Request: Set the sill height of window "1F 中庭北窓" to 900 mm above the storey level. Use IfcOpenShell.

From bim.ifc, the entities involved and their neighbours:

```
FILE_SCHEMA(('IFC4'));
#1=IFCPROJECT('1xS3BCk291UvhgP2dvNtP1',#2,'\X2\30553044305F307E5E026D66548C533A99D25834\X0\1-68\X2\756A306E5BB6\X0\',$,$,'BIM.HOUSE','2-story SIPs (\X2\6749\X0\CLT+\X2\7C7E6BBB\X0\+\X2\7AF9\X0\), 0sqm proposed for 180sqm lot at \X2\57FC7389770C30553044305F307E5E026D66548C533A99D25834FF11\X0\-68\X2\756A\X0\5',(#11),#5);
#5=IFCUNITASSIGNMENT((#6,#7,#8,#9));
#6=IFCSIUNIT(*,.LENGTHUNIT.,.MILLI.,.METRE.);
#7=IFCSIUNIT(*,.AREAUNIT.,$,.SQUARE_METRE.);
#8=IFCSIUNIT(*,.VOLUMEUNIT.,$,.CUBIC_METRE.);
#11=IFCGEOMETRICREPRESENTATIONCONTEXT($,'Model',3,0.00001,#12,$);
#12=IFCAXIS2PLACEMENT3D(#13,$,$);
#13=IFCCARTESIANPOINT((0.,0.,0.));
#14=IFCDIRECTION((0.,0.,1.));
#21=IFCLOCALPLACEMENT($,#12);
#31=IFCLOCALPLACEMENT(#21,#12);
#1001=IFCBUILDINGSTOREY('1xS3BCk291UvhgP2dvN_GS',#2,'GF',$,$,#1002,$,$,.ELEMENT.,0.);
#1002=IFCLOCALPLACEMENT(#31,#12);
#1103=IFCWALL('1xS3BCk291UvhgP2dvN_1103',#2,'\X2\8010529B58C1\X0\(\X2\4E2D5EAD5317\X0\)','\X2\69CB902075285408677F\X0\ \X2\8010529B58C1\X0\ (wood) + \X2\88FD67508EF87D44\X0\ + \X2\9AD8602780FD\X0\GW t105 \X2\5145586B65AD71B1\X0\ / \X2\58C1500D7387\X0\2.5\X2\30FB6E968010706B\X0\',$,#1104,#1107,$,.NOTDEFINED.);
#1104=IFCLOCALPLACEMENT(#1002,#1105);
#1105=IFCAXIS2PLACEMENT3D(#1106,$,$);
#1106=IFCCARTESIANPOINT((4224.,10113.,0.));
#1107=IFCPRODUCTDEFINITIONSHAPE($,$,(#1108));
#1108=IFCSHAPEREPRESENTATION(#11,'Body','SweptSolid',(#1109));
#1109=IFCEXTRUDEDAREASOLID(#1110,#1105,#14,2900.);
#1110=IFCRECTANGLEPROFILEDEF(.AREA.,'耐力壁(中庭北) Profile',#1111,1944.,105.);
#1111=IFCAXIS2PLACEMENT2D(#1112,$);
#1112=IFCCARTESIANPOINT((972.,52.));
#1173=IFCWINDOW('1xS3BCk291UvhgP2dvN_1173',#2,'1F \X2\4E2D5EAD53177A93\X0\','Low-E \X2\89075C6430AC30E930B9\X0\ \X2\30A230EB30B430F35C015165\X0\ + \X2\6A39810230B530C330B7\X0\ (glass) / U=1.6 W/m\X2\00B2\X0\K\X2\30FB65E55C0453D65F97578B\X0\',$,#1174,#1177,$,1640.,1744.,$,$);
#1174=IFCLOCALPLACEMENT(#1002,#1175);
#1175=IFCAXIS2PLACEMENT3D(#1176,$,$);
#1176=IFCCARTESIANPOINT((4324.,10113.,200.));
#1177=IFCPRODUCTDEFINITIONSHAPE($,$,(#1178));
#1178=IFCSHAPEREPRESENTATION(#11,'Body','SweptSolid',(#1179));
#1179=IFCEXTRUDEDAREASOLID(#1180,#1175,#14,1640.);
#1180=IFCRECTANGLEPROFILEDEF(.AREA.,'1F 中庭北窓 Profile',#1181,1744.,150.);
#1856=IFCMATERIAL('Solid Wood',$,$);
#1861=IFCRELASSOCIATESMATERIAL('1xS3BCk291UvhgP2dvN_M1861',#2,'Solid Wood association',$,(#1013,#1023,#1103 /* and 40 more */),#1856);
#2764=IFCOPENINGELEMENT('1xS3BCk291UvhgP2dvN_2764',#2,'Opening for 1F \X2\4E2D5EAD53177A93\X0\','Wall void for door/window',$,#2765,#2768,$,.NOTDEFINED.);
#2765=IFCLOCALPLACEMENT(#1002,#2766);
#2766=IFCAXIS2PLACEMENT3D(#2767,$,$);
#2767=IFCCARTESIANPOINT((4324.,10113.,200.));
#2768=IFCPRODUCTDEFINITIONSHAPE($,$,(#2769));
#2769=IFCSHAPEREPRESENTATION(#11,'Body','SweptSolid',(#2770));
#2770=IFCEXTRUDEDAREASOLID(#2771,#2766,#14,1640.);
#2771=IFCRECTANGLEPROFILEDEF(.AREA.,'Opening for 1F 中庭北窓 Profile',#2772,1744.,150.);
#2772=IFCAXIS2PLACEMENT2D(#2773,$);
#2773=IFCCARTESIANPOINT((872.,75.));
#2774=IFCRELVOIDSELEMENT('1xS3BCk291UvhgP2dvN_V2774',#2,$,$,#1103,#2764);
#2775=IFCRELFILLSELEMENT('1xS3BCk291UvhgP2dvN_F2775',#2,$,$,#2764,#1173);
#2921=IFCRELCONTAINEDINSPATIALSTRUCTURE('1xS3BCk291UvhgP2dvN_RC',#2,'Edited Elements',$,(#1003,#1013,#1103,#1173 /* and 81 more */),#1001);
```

```python
import numpy as np
import ifcopenshell
import ifcopenshell.api.geometry
import ifcopenshell.geom
import ifcopenshell.util.element
import ifcopenshell.util.placement
import ifcopenshell.util.shape
import ifcopenshell.util.unit

model = ifcopenshell.open("bim.ifc")
unit_scale = ifcopenshell.util.unit.calculate_unit_scale(model)

window = model.by_guid("1xS3BCk291UvhgP2dvN_1173")
opening = window.FillsVoids[0].RelatingOpeningElement
storey = ifcopenshell.util.element.get_container(window, ifc_class="IfcBuildingStorey")
level = ifcopenshell.util.placement.get_local_placement(storey.ObjectPlacement)[2, 3]

# The opening's origin need not be at the sill, so measure its lowest point.
shape = ifcopenshell.geom.create_shape(ifcopenshell.geom.settings(), opening)
bottom = ifcopenshell.util.shape.get_shape_bottom_elevation(shape, shape.geometry) / unit_scale
dz = level + 0.9 / unit_scale - bottom

shift = np.array([0.0, 0.0, dz])
# The window is not placed relative to its opening, so move both.
for product in (opening, window):
    matrix = ifcopenshell.util.placement.get_local_placement(product.ObjectPlacement)
    matrix[:3, 3] += shift
    ifcopenshell.api.geometry.edit_object_placement(model, product=product, matrix=matrix, is_si=False)

print(f"moved by {dz * unit_scale:+.3f} m")

model.write("bim_updated.ifc")
```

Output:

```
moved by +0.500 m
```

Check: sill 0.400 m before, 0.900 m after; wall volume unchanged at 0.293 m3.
